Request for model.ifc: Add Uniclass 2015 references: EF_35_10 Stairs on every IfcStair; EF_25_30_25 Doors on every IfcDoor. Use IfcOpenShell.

First a look at what the model holds.

```python
import ifcopenshell

model = ifcopenshell.open("model.ifc")
print(model.schema)
print("classifications:", [c.Name for c in model.by_type("IfcClassification")])
for ifc_class in ("IfcDoor", "IfcRoof", "IfcStair", "IfcWall", "IfcWindow"):
    print(ifc_class, len(model.by_type(ifc_class)))
```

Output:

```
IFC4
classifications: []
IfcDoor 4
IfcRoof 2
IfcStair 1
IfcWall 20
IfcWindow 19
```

```python
import ifcopenshell
import ifcopenshell.api.classification

model = ifcopenshell.open("model.ifc")

system = ifcopenshell.api.classification.add_classification(model, classification="Uniclass 2015")

codes = {
    "IfcStair": ("EF_35_10", "Stairs"),
    "IfcDoor": ("EF_25_30_25", "Doors"),
}
for ifc_class, (code, name) in codes.items():
    products = model.by_type(ifc_class)
    ifcopenshell.api.classification.add_reference(
        model, products=products, classification=system, identification=code, name=name
    )
    print(code, len(products))

model.write("model_updated.ifc")
```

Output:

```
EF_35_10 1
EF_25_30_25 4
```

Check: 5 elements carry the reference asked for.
